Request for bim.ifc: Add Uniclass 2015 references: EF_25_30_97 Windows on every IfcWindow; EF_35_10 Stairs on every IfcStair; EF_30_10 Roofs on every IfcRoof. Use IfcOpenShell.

First a look at what the model holds.

```python
import ifcopenshell

model = ifcopenshell.open("bim.ifc")
print(model.schema)
print("classifications:", [c.Name for c in model.by_type("IfcClassification")])
for ifc_class in ("IfcDoor", "IfcRoof", "IfcStair", "IfcWall", "IfcWindow"):
    print(ifc_class, len(model.by_type(ifc_class)))
```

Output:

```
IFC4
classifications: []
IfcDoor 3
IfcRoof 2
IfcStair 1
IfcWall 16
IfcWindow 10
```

```python
import ifcopenshell
import ifcopenshell.api.classification

model = ifcopenshell.open("bim.ifc")

system = ifcopenshell.api.classification.add_classification(model, classification="Uniclass 2015")

codes = {
    "IfcWindow": ("EF_25_30_97", "Windows"),
    "IfcStair": ("EF_35_10", "Stairs"),
    "IfcRoof": ("EF_30_10", "Roofs"),
}
for ifc_class, (code, name) in codes.items():
    products = model.by_type(ifc_class)
    ifcopenshell.api.classification.add_reference(
        model, products=products, classification=system, identification=code, name=name
    )
    print(code, len(products))

model.write("bim_rev.ifc")
```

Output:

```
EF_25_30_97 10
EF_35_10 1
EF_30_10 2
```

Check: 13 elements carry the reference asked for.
